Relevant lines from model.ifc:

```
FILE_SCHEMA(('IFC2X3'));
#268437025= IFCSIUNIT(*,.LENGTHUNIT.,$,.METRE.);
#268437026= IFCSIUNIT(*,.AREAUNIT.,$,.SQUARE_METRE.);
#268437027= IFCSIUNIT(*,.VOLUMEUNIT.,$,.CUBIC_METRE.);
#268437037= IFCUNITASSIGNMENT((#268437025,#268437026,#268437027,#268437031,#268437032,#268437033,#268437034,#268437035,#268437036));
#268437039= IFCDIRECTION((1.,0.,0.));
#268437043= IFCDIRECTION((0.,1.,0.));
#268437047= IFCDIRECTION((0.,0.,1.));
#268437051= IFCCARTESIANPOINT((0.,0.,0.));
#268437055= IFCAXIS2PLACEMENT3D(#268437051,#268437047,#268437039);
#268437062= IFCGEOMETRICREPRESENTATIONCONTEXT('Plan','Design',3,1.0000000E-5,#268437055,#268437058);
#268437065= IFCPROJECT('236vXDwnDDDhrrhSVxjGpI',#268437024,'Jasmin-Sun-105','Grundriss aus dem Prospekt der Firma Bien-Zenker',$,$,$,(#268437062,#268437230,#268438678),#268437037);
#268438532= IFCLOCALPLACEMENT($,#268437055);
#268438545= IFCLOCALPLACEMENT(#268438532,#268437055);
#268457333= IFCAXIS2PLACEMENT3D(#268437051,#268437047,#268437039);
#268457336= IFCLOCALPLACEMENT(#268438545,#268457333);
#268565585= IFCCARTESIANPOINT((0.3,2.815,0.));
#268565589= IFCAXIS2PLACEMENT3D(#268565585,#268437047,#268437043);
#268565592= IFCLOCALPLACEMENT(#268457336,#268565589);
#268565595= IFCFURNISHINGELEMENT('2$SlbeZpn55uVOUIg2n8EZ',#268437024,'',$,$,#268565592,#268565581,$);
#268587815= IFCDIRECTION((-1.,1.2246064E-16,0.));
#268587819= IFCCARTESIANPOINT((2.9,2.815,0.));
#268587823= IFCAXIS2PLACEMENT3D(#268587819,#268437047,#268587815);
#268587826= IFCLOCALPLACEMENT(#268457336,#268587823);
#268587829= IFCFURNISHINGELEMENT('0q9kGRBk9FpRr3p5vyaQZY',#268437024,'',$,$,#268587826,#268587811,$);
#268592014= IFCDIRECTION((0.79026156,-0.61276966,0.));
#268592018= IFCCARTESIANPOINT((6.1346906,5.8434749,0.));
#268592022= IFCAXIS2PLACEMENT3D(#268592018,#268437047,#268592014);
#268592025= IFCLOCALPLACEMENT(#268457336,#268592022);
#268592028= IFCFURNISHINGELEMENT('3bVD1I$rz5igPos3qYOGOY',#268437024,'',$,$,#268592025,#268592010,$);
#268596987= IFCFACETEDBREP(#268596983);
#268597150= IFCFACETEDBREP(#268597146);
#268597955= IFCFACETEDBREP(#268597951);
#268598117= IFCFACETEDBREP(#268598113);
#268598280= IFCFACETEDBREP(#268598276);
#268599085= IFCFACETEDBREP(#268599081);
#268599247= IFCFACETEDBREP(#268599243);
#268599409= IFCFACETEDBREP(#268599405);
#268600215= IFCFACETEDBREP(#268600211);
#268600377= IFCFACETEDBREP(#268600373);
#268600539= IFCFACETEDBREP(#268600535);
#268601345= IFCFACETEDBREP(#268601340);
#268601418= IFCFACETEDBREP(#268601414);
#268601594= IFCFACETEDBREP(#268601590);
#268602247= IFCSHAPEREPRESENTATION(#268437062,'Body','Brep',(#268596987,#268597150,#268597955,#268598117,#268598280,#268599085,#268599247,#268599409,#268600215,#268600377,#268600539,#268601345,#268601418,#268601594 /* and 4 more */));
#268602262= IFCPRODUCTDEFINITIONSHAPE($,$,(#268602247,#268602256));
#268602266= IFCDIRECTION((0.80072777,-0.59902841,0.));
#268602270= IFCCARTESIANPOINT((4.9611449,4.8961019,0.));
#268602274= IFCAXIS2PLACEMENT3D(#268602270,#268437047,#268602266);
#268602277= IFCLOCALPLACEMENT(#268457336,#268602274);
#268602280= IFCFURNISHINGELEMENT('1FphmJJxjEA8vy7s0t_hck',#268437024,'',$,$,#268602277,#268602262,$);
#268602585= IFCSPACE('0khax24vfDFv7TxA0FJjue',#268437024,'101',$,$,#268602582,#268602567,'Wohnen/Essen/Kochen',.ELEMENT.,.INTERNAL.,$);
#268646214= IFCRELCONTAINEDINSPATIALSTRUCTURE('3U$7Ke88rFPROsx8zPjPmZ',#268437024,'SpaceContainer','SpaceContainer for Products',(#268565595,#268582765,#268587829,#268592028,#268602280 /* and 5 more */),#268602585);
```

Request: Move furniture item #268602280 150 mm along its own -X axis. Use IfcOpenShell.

```python
import ifcopenshell
import ifcopenshell.api.geometry
import ifcopenshell.util.placement
import ifcopenshell.util.unit

model = ifcopenshell.open("model.ifc")
unit_scale = ifcopenshell.util.unit.calculate_unit_scale(model)

item = model.by_guid("1FphmJJxjEA8vy7s0t_hck")
matrix = ifcopenshell.util.placement.get_local_placement(item.ObjectPlacement)
matrix[:3, 3] -= matrix[:3, 0] * 0.15 / unit_scale
ifcopenshell.api.geometry.edit_object_placement(model, product=item, matrix=matrix, is_si=False)

print(ifcopenshell.util.placement.get_local_placement(item.ObjectPlacement).round(3) + 0.0)

model.write("model_v2.ifc")
```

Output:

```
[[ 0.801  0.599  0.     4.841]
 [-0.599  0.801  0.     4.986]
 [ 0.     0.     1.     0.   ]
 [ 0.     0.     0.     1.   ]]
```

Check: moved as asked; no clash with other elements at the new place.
